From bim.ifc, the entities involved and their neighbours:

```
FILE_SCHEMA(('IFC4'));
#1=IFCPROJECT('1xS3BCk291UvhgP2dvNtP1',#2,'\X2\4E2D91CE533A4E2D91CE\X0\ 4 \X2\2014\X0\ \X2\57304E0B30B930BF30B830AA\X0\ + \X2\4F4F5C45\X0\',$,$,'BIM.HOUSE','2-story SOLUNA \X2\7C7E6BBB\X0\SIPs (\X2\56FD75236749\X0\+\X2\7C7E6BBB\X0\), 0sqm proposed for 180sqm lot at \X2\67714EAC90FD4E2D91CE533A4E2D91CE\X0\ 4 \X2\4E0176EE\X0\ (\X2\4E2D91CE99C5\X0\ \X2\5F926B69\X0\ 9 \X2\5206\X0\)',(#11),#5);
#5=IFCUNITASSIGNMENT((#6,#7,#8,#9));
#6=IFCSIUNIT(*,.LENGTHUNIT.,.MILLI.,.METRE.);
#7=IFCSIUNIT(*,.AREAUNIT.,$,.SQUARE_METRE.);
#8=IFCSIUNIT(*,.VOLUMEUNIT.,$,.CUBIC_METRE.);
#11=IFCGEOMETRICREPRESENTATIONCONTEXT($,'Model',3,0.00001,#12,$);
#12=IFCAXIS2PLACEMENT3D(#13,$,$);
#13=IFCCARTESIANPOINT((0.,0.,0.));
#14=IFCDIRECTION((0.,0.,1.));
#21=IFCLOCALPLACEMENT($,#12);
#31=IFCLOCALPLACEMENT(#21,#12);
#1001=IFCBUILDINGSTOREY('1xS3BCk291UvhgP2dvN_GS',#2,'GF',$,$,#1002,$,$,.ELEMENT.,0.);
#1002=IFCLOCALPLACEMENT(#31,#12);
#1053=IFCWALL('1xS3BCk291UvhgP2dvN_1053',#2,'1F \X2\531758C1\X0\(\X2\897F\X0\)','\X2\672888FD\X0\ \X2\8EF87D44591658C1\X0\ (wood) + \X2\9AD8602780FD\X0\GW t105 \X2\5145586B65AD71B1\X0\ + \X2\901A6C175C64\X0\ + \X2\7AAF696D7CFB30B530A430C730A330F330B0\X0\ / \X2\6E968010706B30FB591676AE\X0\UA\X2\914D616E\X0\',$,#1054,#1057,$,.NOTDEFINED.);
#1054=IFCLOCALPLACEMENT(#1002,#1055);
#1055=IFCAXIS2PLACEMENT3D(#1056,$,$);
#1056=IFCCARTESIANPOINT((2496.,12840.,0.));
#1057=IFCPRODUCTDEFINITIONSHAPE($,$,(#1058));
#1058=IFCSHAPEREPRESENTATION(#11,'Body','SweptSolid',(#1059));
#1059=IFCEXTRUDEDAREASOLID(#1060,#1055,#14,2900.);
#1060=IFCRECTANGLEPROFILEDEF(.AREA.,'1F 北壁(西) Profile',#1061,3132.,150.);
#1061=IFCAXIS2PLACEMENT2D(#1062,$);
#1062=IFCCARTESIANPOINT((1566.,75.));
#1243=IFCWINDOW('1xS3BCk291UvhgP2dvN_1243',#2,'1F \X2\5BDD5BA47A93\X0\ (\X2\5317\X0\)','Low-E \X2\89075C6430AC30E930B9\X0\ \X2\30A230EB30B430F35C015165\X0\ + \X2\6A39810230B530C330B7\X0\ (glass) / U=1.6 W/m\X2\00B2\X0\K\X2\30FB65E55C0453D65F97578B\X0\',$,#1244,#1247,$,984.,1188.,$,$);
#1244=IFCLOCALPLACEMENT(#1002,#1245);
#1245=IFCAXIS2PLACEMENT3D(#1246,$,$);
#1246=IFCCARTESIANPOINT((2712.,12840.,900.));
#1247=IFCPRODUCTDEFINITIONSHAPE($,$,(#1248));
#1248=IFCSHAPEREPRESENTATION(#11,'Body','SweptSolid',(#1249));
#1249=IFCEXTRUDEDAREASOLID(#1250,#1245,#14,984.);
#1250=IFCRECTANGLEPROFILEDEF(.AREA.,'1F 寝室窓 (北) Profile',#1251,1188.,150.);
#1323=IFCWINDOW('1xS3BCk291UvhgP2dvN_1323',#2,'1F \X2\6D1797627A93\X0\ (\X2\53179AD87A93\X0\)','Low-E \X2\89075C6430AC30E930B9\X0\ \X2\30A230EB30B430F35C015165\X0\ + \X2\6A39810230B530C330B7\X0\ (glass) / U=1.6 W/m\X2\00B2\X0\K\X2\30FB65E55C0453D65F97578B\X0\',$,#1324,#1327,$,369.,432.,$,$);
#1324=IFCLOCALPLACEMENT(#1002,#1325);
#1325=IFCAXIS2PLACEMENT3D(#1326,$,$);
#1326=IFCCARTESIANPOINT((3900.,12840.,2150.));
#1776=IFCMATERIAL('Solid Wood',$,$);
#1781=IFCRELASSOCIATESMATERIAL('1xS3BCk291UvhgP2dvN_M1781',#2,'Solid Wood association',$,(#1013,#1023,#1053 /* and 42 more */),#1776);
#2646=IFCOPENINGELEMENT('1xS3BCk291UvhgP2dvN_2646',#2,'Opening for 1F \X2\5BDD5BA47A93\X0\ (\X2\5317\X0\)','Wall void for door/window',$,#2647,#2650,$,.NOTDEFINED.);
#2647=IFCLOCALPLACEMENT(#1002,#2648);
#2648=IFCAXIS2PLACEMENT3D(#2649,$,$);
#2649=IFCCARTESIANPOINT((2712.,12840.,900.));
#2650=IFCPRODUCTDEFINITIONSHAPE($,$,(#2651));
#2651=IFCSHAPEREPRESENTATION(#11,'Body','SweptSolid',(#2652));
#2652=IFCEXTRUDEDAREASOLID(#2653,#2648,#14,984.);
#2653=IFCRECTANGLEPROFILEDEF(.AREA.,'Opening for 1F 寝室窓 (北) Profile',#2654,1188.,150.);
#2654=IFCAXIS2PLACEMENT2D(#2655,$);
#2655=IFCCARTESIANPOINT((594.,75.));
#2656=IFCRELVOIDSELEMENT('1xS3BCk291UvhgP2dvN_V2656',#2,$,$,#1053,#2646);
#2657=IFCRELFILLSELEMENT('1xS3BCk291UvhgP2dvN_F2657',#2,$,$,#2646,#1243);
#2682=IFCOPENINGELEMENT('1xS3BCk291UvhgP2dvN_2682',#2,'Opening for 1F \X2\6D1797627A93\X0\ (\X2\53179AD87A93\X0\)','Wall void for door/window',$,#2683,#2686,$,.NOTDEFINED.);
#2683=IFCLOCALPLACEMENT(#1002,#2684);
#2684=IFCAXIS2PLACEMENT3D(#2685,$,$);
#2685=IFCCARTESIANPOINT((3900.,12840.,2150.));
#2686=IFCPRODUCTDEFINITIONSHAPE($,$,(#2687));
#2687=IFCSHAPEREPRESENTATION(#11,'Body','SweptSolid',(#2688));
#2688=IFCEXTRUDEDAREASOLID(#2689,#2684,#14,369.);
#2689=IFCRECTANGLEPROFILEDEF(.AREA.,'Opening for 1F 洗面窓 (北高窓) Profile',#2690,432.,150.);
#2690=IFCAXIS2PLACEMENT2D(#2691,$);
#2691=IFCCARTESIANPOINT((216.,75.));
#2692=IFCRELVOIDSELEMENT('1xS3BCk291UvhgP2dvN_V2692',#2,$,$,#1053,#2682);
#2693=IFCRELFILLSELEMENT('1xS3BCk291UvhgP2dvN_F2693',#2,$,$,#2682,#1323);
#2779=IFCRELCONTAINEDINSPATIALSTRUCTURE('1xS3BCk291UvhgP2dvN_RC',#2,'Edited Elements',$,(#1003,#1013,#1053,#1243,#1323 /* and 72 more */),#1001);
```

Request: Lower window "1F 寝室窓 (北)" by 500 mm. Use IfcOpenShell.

```python
import numpy as np
import ifcopenshell
import ifcopenshell.api.geometry
import ifcopenshell.util.placement
import ifcopenshell.util.unit

model = ifcopenshell.open("bim.ifc")
unit_scale = ifcopenshell.util.unit.calculate_unit_scale(model)

window = model.by_guid("1xS3BCk291UvhgP2dvN_1243")
opening = window.FillsVoids[0].RelatingOpeningElement
dz = -0.5 / unit_scale

shift = np.array([0.0, 0.0, dz])
# The window is not placed relative to its opening, so move both.
for product in (opening, window):
    matrix = ifcopenshell.util.placement.get_local_placement(product.ObjectPlacement)
    matrix[:3, 3] += shift
    ifcopenshell.api.geometry.edit_object_placement(model, product=product, matrix=matrix, is_si=False)

print(f"moved by {dz * unit_scale:+.3f} m")

model.write("bim_updated.ifc")
```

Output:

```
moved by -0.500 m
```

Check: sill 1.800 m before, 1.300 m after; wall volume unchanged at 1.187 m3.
